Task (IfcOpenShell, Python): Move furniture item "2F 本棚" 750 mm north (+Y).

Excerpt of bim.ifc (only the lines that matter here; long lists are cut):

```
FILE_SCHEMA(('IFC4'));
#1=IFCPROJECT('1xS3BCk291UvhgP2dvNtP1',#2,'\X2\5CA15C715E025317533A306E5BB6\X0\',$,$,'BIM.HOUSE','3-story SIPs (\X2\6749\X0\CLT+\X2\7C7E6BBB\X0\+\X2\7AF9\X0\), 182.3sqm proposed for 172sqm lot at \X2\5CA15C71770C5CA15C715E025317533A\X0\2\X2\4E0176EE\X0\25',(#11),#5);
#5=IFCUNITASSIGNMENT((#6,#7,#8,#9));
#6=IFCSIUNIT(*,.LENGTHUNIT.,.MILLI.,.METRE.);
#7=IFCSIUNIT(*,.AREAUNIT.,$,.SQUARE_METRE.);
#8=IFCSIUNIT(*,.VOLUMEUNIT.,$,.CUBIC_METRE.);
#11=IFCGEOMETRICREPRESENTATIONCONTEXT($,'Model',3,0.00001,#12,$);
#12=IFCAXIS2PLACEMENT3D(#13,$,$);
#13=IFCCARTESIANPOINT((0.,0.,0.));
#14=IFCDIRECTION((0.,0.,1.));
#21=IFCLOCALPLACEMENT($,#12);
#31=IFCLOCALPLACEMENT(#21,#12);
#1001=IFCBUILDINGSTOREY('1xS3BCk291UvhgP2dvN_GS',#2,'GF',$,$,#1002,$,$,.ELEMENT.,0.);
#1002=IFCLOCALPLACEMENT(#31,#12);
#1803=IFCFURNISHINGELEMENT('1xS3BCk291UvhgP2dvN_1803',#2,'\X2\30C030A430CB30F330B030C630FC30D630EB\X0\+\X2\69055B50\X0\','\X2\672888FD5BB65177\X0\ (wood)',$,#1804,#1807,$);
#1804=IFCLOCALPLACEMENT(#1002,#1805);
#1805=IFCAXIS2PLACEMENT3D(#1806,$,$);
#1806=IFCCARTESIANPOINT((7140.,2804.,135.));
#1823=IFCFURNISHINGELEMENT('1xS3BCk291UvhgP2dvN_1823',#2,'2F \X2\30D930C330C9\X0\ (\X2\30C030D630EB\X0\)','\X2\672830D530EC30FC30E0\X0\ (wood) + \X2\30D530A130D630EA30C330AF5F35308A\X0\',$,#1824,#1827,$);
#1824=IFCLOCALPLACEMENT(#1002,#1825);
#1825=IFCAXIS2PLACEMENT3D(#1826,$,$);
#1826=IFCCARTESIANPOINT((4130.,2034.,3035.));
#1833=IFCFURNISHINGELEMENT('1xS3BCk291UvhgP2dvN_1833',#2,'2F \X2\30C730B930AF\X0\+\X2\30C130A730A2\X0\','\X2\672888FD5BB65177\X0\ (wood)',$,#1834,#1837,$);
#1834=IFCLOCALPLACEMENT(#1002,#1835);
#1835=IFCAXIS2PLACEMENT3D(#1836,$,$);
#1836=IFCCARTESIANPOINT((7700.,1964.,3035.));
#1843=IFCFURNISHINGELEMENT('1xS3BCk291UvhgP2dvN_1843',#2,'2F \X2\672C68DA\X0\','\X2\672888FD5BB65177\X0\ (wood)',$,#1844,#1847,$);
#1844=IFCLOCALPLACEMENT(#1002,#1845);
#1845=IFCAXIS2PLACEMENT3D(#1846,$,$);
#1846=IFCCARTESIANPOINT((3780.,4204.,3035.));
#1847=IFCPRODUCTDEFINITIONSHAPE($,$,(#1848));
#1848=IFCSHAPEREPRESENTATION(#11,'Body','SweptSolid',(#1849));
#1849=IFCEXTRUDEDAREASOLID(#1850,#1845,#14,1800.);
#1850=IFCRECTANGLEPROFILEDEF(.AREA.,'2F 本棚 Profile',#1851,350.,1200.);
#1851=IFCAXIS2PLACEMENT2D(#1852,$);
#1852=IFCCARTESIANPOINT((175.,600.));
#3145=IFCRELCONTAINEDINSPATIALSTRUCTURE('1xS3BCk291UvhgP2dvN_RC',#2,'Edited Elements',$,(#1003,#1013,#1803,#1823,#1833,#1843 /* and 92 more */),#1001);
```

```python
import ifcopenshell
import ifcopenshell.api.geometry
import ifcopenshell.util.placement
import ifcopenshell.util.unit

model = ifcopenshell.open("bim.ifc")
unit_scale = ifcopenshell.util.unit.calculate_unit_scale(model)

item = model.by_id(1843)
matrix = ifcopenshell.util.placement.get_local_placement(item.ObjectPlacement)
matrix[1, 3] += 0.75 / unit_scale
ifcopenshell.api.geometry.edit_object_placement(model, product=item, matrix=matrix, is_si=False)

print(ifcopenshell.util.placement.get_local_placement(item.ObjectPlacement).round(3) + 0.0)

model.write("bim-out.ifc")
```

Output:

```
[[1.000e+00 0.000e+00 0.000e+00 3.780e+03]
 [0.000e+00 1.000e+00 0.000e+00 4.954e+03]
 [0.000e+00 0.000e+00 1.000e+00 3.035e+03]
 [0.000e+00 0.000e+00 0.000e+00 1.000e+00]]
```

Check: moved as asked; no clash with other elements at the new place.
